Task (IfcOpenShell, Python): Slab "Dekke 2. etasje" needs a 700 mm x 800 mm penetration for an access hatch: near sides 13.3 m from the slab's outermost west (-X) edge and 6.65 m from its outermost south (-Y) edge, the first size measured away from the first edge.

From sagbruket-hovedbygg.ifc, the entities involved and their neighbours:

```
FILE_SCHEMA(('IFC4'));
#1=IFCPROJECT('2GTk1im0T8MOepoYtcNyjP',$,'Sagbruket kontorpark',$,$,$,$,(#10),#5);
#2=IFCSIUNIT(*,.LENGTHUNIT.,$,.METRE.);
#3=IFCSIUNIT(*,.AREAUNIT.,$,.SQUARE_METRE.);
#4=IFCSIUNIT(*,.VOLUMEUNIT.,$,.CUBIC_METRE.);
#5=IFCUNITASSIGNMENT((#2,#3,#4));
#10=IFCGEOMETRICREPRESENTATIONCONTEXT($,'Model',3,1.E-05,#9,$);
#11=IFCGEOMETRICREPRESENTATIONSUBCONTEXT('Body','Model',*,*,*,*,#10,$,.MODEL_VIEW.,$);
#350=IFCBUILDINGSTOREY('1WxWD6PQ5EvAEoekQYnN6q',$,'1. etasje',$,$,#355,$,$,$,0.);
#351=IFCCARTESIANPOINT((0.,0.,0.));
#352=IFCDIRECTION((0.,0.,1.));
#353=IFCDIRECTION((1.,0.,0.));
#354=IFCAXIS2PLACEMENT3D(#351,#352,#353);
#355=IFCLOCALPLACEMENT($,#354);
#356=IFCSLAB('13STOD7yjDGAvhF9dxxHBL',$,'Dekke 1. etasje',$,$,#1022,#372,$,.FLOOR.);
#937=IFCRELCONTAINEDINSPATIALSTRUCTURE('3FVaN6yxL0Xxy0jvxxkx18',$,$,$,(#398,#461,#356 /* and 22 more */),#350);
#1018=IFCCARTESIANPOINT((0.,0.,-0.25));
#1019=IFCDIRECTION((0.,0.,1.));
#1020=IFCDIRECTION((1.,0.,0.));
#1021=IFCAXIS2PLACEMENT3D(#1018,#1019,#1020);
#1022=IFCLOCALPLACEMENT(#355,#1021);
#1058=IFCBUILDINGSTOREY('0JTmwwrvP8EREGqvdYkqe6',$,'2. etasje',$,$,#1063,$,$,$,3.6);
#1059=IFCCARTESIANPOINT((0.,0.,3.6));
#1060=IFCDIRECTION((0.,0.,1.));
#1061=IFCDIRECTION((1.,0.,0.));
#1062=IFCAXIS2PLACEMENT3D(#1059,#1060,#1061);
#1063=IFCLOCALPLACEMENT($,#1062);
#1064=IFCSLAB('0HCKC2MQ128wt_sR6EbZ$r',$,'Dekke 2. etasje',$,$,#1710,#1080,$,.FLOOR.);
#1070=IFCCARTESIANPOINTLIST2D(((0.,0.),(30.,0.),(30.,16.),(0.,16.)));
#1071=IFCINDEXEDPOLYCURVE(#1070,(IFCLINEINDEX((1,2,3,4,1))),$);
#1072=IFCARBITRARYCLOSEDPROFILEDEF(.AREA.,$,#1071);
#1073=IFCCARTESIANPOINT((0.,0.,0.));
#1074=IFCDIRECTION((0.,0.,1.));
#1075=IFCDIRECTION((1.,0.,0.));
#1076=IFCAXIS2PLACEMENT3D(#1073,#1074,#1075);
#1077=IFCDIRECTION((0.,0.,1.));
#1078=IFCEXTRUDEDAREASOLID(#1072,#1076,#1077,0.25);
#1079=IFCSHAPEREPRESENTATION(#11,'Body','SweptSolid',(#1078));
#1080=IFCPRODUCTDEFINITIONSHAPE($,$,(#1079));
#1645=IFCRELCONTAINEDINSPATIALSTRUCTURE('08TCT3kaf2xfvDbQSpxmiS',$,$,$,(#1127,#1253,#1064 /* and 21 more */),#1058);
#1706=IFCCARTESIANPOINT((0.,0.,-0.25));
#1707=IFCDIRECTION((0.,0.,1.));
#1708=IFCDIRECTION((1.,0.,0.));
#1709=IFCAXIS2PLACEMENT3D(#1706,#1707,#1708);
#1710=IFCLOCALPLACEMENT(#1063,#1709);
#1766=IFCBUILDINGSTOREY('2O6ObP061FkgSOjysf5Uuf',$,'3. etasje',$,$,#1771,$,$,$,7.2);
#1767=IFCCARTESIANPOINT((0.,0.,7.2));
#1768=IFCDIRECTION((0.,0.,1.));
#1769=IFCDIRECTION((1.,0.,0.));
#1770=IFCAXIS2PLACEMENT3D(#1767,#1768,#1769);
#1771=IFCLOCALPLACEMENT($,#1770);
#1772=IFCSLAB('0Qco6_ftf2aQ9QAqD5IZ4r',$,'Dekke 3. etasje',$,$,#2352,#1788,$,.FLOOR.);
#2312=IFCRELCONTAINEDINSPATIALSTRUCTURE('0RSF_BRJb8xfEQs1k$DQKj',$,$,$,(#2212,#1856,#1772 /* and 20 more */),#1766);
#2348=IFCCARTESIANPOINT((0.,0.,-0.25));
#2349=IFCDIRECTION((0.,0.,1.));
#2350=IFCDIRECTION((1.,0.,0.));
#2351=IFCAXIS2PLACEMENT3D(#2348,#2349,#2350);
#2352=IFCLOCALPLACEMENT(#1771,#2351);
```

```python
import numpy as np
import ifcopenshell
import ifcopenshell.api.feature
import ifcopenshell.api.geometry
import ifcopenshell.api.root
import ifcopenshell.geom
import ifcopenshell.util.placement
import ifcopenshell.util.representation
import ifcopenshell.util.shape
import ifcopenshell.util.unit

model = ifcopenshell.open("sagbruket-hovedbygg.ifc")
unit_scale = ifcopenshell.util.unit.calculate_unit_scale(model)
settings = ifcopenshell.geom.settings()


def volume(element):
    """Net volume in cubic metres, openings subtracted."""
    shape = ifcopenshell.geom.create_shape(settings, element)
    return ifcopenshell.util.shape.get_volume(shape.geometry)


slab = model.by_guid("0HCKC2MQ128wt_sR6EbZ$r")
before = volume(slab)

# Extent in the slab's own axes, in metres. The edges named are its -X and -Y sides.
slab_shape = ifcopenshell.geom.create_shape(settings, slab)
vertices = ifcopenshell.util.shape.get_vertices(slab_shape.geometry)
x_min, y_min, bottom = vertices.min(axis=0)
top = vertices[:, 2].max()

opening = ifcopenshell.api.root.create_entity(model, ifc_class="IfcOpeningElement", name="Access hatch opening", predefined_type="OPENING")
context = ifcopenshell.util.representation.get_context(model, "Model", "Body", "MODEL_VIEW")
width, depth = 0.7, 0.8
outline = [(0.0, 0.0), (width, 0.0), (width, depth), (0.0, depth), (0.0, 0.0)]
# Overshoot both faces by 50 mm so the cut is clean.
shape = ifcopenshell.api.geometry.add_slab_representation(
    model, context=context, depth=top - bottom + 0.1, polyline=outline
)
ifcopenshell.api.geometry.assign_representation(model, product=opening, representation=shape)

matrix = ifcopenshell.util.placement.get_local_placement(slab.ObjectPlacement)
matrix[:, 3] = matrix @ np.append(np.array([x_min + 13.3, y_min + 6.65, bottom - 0.05]) / unit_scale, 1.0)
ifcopenshell.api.geometry.edit_object_placement(model, product=opening, matrix=matrix, is_si=False)
ifcopenshell.api.feature.add_feature(model, feature=opening, element=slab)

after = volume(slab)

print(f"slab volume {before:.3f} -> {after:.3f} m3")

model.write("sagbruket-hovedbygg-out.ifc")
```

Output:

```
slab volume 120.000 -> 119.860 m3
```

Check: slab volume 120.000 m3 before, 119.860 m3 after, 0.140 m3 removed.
